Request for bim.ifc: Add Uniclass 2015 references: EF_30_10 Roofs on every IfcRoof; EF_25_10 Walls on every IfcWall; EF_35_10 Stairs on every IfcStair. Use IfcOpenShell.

First a look at what the model holds.

```python
import ifcopenshell

model = ifcopenshell.open("bim.ifc")
print(model.schema)
print("classifications:", [c.Name for c in model.by_type("IfcClassification")])
for ifc_class in ("IfcDoor", "IfcRoof", "IfcStair", "IfcWall", "IfcWindow"):
    print(ifc_class, len(model.by_type(ifc_class)))
```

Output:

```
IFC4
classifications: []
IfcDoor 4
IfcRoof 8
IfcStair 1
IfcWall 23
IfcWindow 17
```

```python
import ifcopenshell
import ifcopenshell.api.classification

model = ifcopenshell.open("bim.ifc")

system = ifcopenshell.api.classification.add_classification(model, classification="Uniclass 2015")

codes = {
    "IfcRoof": ("EF_30_10", "Roofs"),
    "IfcWall": ("EF_25_10", "Walls"),
    "IfcStair": ("EF_35_10", "Stairs"),
}
for ifc_class, (code, name) in codes.items():
    products = model.by_type(ifc_class)
    ifcopenshell.api.classification.add_reference(
        model, products=products, classification=system, identification=code, name=name
    )
    print(code, len(products))

model.write("bim_updated.ifc")
```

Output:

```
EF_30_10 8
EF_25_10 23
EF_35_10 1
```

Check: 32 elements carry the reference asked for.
